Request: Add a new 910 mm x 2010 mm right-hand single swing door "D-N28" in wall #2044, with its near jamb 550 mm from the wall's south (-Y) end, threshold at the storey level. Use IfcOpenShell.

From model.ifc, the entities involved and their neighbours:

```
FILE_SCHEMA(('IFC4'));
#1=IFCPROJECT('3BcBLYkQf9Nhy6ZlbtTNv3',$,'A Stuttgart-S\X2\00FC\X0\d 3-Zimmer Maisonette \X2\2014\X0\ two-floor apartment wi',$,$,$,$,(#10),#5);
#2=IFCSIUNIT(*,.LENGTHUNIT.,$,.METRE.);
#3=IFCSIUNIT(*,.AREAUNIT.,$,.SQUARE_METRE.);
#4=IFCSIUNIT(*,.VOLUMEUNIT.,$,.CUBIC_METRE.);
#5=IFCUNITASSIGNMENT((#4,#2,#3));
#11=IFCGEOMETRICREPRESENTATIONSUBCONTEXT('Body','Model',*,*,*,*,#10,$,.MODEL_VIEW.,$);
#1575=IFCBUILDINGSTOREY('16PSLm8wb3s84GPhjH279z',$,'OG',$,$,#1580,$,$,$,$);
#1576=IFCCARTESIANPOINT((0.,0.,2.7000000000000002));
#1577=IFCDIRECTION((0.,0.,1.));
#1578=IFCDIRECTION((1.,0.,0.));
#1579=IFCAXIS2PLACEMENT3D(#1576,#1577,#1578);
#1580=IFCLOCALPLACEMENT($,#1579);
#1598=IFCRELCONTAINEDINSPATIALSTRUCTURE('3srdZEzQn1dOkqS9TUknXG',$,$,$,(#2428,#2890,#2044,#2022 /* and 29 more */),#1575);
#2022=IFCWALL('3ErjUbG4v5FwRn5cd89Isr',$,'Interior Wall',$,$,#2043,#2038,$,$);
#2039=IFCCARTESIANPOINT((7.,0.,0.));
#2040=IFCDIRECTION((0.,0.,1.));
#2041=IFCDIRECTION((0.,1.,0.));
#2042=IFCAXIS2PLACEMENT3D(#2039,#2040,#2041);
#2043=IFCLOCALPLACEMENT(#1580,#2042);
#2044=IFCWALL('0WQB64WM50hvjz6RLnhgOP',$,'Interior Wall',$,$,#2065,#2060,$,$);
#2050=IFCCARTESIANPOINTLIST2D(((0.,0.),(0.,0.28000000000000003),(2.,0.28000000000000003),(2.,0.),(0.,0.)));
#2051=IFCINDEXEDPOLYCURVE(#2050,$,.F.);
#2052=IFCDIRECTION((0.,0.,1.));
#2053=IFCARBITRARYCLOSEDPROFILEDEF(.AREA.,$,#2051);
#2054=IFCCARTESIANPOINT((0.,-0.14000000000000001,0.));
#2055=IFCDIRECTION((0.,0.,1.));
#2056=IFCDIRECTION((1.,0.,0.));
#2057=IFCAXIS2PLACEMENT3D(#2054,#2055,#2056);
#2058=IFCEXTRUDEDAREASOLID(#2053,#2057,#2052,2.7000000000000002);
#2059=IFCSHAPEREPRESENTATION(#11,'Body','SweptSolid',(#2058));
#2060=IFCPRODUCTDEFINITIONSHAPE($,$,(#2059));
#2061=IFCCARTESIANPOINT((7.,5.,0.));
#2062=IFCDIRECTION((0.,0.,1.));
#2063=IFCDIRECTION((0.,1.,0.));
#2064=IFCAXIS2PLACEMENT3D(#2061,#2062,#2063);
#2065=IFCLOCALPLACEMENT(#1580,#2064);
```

```python
import numpy as np
import ifcopenshell
import ifcopenshell.api.feature
import ifcopenshell.api.geometry
import ifcopenshell.api.root
import ifcopenshell.api.spatial
import ifcopenshell.geom
import ifcopenshell.util.element
import ifcopenshell.util.placement
import ifcopenshell.util.representation
import ifcopenshell.util.shape
import ifcopenshell.util.unit

model = ifcopenshell.open("model.ifc")
unit_scale = ifcopenshell.util.unit.calculate_unit_scale(model)
settings = ifcopenshell.geom.settings()


def volume(element):
    """Net volume in cubic metres, openings subtracted."""
    shape = ifcopenshell.geom.create_shape(settings, element)
    return ifcopenshell.util.shape.get_volume(shape.geometry)


wall = model.by_guid("0WQB64WM50hvjz6RLnhgOP")
storey = ifcopenshell.util.element.get_container(wall, ifc_class="IfcBuildingStorey")
context = ifcopenshell.util.representation.get_context(model, "Model", "Body", "MODEL_VIEW")
before = volume(wall)

width, height, from_end, sill = 0.91, 2.01, 0.55, 0.0  # metres

# The wall runs along its own X axis, and the end named is its -X end.
wall_shape = ifcopenshell.geom.create_shape(settings, wall)
x, y, z = ifcopenshell.util.shape.get_vertices(wall_shape.geometry).T
start = x.min() + from_end
face, thickness = float(y.min()), float(y.max() - y.min())
wall_matrix = ifcopenshell.util.placement.get_local_placement(wall.ObjectPlacement)
level = ifcopenshell.util.placement.get_local_placement(storey.ObjectPlacement)[2, 3]


def in_wall(x, y):
    """Placement at x, y metres in the wall's axes, at sill height."""
    matrix = wall_matrix.copy()
    matrix[:, 3] = wall_matrix @ np.array([x / unit_scale, y / unit_scale, 0.0, 1.0])
    matrix[2, 3] = level + sill / unit_scale
    return matrix


# Opening: a box that overshoots both wall faces by 50 mm.
opening = ifcopenshell.api.root.create_entity(model, ifc_class="IfcOpeningElement", predefined_type="OPENING")
box = ifcopenshell.api.geometry.add_wall_representation(
    model, context=context, length=width, height=height, thickness=thickness + 0.1
)
ifcopenshell.api.geometry.assign_representation(model, product=opening, representation=box)
ifcopenshell.api.geometry.edit_object_placement(model, product=opening, matrix=in_wall(start, face - 0.05), is_si=False)
ifcopenshell.api.feature.add_feature(model, feature=opening, element=wall)

door = ifcopenshell.api.root.create_entity(model, ifc_class="IfcDoor", name="D-N28", predefined_type="DOOR")
door.OverallWidth, door.OverallHeight = width / unit_scale, height / unit_scale
door.OperationType = "SINGLE_SWING_RIGHT"
body = ifcopenshell.api.geometry.add_door_representation(
    model,
    context=context,
    overall_width=door.OverallWidth,
    overall_height=door.OverallHeight,
    operation_type="SINGLE_SWING_RIGHT",
    lining_properties={"LiningDepth": thickness / unit_scale, "ThresholdDepth": thickness / unit_scale},
)
ifcopenshell.api.geometry.assign_representation(model, product=door, representation=body)
ifcopenshell.api.spatial.assign_container(model, products=[door], relating_structure=storey)
ifcopenshell.api.feature.add_filling(model, opening=opening, element=door)

# The lining spans the wall, so the door starts at the wall face.
ifcopenshell.api.geometry.edit_object_placement(model, product=door, matrix=in_wall(start, face), is_si=False)

after = volume(wall)

print(f"wall volume {before:.3f} -> {after:.3f} m3")

model.write("model_edited.ifc")
```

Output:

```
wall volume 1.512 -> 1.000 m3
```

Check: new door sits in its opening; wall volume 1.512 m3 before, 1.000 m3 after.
